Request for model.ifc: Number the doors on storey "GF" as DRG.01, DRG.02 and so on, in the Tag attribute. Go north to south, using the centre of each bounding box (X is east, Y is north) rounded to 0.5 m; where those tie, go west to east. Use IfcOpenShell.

First a look at what the model holds.

```python
import ifcopenshell
import ifcopenshell.util.element
import ifcopenshell.util.placement

model = ifcopenshell.open("model.ifc")
print(model.schema)
storey = next(s for s in model.by_type("IfcBuildingStorey") if s.Name == "GF")
doors = [e for e in ifcopenshell.util.element.get_decomposition(storey) if e.is_a("IfcDoor")]
for e in sorted(doors, key=lambda e: e.id()):
    origin = ifcopenshell.util.placement.get_local_placement(e.ObjectPlacement)[:3, 3]
    print(e.id(), e.Tag, e.Name, origin.round(2) + 0.0, sep=" | ")
```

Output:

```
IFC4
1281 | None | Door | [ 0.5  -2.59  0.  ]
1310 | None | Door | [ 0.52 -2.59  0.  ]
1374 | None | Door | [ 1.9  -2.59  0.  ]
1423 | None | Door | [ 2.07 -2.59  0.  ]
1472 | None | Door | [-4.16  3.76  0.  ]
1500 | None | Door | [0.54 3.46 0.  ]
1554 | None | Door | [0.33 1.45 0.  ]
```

```python
import ifcopenshell
import ifcopenshell.geom
import ifcopenshell.util.element
import ifcopenshell.util.shape

model = ifcopenshell.open("model.ifc")
settings = ifcopenshell.geom.settings()
settings.set("use-world-coords", True)


def centre(element):
    shape = ifcopenshell.geom.create_shape(settings, element)
    return ifcopenshell.util.shape.get_bbox_centroid(shape.geometry)


storey = next(s for s in model.by_type("IfcBuildingStorey") if s.Name == "GF")
doors = [e for e in ifcopenshell.util.element.get_decomposition(storey) if e.is_a("IfcDoor")]

# Insertion points can sit at a corner or the storey origin, so sort by the geometry (in metres).
centres = {e: centre(e) for e in doors}
doors.sort(key=lambda e: (-round(centres[e][1] / 0.5), centres[e][0]))

for i, e in enumerate(doors, start=1):
    number = f"DRG.{i:02d}"
    e.Tag = number
    print(e.id(), number)

model.write("model-out.ifc")
```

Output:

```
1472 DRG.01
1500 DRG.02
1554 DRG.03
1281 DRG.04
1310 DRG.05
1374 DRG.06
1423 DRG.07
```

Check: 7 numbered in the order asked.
